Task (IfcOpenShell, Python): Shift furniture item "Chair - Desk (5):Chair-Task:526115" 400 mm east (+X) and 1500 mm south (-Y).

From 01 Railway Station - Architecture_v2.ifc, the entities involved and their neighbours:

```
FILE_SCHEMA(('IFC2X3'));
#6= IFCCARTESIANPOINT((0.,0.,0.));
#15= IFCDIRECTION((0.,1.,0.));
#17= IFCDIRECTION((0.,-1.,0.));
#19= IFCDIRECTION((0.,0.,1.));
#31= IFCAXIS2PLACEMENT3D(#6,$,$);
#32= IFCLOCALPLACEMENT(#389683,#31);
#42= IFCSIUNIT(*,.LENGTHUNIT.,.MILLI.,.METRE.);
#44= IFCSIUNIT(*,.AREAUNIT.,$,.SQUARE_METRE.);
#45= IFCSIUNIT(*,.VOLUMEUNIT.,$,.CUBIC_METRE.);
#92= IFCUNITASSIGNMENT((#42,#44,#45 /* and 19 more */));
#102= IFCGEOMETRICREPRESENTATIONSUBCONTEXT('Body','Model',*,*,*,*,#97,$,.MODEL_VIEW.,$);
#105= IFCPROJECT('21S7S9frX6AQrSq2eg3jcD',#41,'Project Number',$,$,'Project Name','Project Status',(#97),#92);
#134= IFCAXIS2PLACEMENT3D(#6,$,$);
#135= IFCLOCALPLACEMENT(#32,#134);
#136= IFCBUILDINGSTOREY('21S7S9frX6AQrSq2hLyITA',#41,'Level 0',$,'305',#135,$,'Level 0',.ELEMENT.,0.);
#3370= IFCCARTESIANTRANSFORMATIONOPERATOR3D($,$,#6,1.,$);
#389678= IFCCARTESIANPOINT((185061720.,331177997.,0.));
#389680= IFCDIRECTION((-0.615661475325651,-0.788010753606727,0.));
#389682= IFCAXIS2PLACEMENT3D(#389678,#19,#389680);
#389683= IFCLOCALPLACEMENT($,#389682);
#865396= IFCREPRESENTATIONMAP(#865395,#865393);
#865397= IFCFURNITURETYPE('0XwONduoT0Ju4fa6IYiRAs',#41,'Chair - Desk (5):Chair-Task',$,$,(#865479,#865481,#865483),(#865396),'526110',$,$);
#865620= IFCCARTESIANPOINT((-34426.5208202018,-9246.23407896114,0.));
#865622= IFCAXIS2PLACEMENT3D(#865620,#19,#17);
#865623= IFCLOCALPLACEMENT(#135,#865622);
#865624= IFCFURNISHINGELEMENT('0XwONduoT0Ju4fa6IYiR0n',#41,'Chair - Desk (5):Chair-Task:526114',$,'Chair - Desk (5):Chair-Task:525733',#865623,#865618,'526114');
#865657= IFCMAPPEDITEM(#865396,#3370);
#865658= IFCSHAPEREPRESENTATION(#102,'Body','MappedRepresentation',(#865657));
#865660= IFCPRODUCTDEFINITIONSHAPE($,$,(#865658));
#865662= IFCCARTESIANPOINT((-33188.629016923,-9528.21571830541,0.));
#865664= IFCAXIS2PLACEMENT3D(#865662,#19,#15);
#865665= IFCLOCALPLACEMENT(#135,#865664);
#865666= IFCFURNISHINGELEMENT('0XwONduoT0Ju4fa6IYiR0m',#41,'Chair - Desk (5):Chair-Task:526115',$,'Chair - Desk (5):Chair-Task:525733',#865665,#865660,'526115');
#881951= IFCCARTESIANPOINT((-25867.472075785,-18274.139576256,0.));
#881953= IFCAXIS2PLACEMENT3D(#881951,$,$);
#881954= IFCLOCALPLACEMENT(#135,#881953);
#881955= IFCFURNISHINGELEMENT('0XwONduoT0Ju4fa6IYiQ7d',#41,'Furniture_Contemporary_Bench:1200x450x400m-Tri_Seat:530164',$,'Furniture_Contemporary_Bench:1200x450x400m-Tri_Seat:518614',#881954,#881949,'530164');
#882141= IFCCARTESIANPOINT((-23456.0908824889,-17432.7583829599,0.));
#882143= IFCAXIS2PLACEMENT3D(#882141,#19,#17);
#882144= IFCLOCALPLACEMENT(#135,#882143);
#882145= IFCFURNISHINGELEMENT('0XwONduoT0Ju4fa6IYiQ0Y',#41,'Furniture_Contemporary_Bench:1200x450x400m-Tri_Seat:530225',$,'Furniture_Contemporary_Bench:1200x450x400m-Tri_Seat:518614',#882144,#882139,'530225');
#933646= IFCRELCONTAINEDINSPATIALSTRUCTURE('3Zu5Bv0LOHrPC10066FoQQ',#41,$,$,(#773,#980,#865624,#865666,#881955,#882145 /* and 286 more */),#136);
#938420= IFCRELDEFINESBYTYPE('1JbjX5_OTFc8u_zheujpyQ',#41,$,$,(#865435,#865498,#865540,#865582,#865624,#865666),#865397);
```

```python
import ifcopenshell
import ifcopenshell.api.geometry
import ifcopenshell.util.placement

model = ifcopenshell.open("01 Railway Station - Architecture_v2.ifc")

item = model.by_guid("0XwONduoT0Ju4fa6IYiR0m")
matrix = ifcopenshell.util.placement.get_local_placement(item.ObjectPlacement)
matrix[0, 3] += 400.0
matrix[1, 3] -= 1500.0
ifcopenshell.api.geometry.edit_object_placement(model, product=item, matrix=matrix, is_si=False)

print(ifcopenshell.util.placement.get_local_placement(item.ObjectPlacement).round(3) + 0.0)

model.write("01 Railway Station - Architecture_v2_rev.ifc")
```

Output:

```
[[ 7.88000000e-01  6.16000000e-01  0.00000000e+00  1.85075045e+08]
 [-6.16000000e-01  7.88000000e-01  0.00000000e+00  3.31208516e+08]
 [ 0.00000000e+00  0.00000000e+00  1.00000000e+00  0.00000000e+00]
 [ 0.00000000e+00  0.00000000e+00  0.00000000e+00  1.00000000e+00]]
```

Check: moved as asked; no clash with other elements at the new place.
